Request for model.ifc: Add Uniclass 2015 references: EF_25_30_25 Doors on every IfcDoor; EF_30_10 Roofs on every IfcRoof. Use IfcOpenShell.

First a look at what the model holds.

```python
import ifcopenshell

model = ifcopenshell.open("model.ifc")
print(model.schema)
print("classifications:", [c.Name for c in model.by_type("IfcClassification")])
for ifc_class in ("IfcDoor", "IfcRoof", "IfcStair", "IfcWall", "IfcWindow"):
    print(ifc_class, len(model.by_type(ifc_class)))
```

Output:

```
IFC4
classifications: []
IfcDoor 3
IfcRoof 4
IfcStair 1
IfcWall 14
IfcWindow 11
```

```python
import ifcopenshell
import ifcopenshell.api.classification

model = ifcopenshell.open("model.ifc")

system = ifcopenshell.api.classification.add_classification(model, classification="Uniclass 2015")

codes = {
    "IfcDoor": ("EF_25_30_25", "Doors"),
    "IfcRoof": ("EF_30_10", "Roofs"),
}
for ifc_class, (code, name) in codes.items():
    products = model.by_type(ifc_class)
    ifcopenshell.api.classification.add_reference(
        model, products=products, classification=system, identification=code, name=name
    )
    print(code, len(products))

model.write("model_updated.ifc")
```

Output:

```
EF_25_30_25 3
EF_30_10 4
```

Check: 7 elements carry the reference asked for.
